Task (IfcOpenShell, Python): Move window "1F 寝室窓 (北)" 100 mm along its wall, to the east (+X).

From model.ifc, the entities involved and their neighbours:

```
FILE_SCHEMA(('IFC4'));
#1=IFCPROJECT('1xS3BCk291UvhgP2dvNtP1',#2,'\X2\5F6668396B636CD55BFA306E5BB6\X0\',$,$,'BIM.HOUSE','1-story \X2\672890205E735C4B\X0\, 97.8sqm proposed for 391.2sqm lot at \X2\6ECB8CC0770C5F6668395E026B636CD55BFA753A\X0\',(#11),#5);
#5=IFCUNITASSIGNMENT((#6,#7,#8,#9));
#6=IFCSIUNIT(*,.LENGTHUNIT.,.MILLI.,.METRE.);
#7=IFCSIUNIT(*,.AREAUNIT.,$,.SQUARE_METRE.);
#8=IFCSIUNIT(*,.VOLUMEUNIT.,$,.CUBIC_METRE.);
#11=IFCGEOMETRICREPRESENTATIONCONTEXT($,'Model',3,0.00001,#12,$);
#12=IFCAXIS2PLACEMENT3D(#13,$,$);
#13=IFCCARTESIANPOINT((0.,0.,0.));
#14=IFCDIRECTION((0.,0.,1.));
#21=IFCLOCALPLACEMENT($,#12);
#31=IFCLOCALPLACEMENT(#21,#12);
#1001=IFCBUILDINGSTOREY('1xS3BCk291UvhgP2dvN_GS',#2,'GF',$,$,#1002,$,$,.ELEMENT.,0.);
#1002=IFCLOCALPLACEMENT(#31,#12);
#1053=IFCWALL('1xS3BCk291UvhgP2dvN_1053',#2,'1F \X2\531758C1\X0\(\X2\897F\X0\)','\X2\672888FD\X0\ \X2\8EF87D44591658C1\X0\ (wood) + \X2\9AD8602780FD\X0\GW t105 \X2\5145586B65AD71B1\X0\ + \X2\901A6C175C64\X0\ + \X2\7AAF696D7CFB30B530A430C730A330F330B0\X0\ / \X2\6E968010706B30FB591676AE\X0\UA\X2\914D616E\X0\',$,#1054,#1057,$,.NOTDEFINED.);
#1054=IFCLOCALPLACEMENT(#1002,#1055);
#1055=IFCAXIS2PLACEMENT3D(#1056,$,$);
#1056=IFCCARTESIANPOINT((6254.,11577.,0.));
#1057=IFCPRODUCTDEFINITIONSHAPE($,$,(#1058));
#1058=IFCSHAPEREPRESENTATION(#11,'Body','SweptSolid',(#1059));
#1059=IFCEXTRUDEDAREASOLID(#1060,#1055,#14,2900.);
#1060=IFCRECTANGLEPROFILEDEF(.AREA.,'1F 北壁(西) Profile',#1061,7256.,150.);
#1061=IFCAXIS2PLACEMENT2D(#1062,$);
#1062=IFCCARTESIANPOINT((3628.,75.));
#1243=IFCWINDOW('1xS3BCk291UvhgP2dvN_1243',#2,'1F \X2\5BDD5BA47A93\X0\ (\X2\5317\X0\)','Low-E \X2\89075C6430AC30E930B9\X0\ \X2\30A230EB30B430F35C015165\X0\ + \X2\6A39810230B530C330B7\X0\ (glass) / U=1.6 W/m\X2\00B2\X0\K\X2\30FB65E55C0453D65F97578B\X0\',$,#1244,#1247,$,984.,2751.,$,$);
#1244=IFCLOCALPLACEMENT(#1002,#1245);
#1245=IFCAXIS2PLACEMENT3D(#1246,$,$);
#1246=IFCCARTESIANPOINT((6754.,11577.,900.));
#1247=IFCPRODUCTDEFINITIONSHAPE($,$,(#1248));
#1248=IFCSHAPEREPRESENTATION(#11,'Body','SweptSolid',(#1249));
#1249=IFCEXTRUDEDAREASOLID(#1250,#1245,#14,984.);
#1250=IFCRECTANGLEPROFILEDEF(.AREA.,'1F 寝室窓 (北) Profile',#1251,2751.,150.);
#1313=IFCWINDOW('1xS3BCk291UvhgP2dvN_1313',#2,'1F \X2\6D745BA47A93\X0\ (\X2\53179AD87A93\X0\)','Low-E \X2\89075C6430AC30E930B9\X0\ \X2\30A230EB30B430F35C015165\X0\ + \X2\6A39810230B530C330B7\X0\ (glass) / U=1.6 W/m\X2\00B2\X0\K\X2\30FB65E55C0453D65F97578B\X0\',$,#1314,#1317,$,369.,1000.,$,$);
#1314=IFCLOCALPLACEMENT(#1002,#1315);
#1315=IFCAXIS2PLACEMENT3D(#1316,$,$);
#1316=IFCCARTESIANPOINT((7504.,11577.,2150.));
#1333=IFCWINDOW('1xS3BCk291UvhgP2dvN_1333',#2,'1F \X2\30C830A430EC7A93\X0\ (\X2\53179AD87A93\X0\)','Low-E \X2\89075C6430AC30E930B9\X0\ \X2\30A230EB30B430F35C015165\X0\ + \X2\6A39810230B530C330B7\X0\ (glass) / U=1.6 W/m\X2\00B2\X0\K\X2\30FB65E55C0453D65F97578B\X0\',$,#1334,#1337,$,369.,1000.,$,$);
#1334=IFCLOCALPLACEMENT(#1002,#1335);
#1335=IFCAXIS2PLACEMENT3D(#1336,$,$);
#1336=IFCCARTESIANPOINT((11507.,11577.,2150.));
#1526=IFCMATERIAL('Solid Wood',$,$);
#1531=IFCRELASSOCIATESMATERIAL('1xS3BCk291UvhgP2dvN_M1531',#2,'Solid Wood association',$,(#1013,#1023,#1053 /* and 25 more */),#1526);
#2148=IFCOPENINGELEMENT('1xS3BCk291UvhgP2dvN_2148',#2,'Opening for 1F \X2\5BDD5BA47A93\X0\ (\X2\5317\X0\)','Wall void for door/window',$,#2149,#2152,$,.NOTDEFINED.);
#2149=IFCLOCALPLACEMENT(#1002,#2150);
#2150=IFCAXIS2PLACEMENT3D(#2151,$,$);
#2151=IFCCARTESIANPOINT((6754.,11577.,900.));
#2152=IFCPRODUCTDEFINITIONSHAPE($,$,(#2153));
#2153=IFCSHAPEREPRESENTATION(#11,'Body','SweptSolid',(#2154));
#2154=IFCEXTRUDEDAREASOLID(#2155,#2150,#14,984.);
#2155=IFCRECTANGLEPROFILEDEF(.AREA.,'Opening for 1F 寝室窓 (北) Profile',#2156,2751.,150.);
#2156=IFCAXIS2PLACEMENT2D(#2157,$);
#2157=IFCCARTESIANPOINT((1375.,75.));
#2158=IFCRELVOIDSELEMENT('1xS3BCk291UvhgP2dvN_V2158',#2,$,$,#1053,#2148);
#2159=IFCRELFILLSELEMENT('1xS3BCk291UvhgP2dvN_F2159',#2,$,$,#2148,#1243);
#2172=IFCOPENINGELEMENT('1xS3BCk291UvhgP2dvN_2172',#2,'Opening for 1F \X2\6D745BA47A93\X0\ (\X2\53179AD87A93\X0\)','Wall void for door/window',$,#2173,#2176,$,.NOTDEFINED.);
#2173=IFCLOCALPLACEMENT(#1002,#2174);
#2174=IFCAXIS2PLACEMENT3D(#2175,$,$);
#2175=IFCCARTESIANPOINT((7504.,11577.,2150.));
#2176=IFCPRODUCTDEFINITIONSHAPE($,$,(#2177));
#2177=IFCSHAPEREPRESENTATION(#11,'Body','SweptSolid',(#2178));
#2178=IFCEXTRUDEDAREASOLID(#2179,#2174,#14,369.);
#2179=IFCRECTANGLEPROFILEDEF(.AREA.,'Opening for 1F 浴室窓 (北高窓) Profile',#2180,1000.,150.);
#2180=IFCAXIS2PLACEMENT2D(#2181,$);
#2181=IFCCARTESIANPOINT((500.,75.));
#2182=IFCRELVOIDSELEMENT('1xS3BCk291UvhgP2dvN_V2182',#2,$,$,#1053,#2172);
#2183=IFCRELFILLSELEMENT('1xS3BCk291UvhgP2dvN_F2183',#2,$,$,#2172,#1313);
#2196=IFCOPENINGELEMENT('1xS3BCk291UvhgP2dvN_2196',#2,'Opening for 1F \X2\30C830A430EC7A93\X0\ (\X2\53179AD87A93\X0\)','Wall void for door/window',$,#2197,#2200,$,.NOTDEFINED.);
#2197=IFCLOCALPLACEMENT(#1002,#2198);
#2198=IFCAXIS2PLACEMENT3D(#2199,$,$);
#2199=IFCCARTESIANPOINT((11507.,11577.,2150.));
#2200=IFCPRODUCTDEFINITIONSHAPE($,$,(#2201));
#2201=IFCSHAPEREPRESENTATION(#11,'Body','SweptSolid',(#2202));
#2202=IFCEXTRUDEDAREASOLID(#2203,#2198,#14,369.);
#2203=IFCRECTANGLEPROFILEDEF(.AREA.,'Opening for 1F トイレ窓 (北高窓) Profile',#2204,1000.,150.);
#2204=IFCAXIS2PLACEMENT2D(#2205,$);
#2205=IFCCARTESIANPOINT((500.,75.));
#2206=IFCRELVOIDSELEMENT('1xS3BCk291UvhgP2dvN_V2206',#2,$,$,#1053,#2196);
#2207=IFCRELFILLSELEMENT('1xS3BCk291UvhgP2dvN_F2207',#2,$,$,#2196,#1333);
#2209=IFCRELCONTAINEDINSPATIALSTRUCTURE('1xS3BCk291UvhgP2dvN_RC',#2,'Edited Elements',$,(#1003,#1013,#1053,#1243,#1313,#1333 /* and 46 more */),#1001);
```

```python
import ifcopenshell
import ifcopenshell.api.geometry
import ifcopenshell.util.placement
import ifcopenshell.util.unit

model = ifcopenshell.open("model.ifc")
unit_scale = ifcopenshell.util.unit.calculate_unit_scale(model)

window = model.by_guid("1xS3BCk291UvhgP2dvN_1243")
opening = window.FillsVoids[0].RelatingOpeningElement
wall = opening.VoidsElements[0].RelatingBuildingElement

wall_matrix = ifcopenshell.util.placement.get_local_placement(wall.ObjectPlacement)
shift = wall_matrix[:3, 0] * 0.1 / unit_scale
before = ifcopenshell.util.placement.get_local_placement(window.ObjectPlacement)[:3, 3].copy()

# The window is not placed relative to its opening, so move both.
for product in (opening, window):
    matrix = ifcopenshell.util.placement.get_local_placement(product.ObjectPlacement)
    matrix[:3, 3] += shift
    ifcopenshell.api.geometry.edit_object_placement(model, product=product, matrix=matrix, is_si=False)

after = ifcopenshell.util.placement.get_local_placement(window.ObjectPlacement)[:3, 3]
print("window moved by", (after - before).round(3) + 0.0)

model.write("model_v2.ifc")
```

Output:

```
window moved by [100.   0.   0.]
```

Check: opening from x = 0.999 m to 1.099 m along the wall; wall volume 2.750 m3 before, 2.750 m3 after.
